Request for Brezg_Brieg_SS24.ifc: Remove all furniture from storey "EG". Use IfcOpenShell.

First a look at what the model holds.

```python
import ifcopenshell
import ifcopenshell.util.element

model = ifcopenshell.open("Brezg_Brieg_SS24.ifc")
print(model.schema)
storey = next(s for s in model.by_type("IfcBuildingStorey") if s.Name == "EG")
furniture = [e for e in ifcopenshell.util.element.get_decomposition(storey) if e.is_a("IfcFurnishingElement")]
seen = {}
for e in furniture:
    element_type = ifcopenshell.util.element.get_type(e)
    name = element_type.Name if element_type not in (None, e) else None
    seen[name] = seen.get(name, 0) + 1
for name, count in sorted(seen.items(), key=str):
    print(count, "x", name)
```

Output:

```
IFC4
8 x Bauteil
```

```python
import ifcopenshell
import ifcopenshell.api.root
import ifcopenshell.util.element

model = ifcopenshell.open("Brezg_Brieg_SS24.ifc")

storey = next(s for s in model.by_type("IfcBuildingStorey") if s.Name == "EG")
furniture = [e for e in ifcopenshell.util.element.get_decomposition(storey) if e.is_a("IfcFurnishingElement")]

for e in furniture:
    ifcopenshell.api.root.remove_product(model, product=e)
print(len(furniture), "removed")

model.write("Brezg_Brieg_SS24_updated.ifc")
```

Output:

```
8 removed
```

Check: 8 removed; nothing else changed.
